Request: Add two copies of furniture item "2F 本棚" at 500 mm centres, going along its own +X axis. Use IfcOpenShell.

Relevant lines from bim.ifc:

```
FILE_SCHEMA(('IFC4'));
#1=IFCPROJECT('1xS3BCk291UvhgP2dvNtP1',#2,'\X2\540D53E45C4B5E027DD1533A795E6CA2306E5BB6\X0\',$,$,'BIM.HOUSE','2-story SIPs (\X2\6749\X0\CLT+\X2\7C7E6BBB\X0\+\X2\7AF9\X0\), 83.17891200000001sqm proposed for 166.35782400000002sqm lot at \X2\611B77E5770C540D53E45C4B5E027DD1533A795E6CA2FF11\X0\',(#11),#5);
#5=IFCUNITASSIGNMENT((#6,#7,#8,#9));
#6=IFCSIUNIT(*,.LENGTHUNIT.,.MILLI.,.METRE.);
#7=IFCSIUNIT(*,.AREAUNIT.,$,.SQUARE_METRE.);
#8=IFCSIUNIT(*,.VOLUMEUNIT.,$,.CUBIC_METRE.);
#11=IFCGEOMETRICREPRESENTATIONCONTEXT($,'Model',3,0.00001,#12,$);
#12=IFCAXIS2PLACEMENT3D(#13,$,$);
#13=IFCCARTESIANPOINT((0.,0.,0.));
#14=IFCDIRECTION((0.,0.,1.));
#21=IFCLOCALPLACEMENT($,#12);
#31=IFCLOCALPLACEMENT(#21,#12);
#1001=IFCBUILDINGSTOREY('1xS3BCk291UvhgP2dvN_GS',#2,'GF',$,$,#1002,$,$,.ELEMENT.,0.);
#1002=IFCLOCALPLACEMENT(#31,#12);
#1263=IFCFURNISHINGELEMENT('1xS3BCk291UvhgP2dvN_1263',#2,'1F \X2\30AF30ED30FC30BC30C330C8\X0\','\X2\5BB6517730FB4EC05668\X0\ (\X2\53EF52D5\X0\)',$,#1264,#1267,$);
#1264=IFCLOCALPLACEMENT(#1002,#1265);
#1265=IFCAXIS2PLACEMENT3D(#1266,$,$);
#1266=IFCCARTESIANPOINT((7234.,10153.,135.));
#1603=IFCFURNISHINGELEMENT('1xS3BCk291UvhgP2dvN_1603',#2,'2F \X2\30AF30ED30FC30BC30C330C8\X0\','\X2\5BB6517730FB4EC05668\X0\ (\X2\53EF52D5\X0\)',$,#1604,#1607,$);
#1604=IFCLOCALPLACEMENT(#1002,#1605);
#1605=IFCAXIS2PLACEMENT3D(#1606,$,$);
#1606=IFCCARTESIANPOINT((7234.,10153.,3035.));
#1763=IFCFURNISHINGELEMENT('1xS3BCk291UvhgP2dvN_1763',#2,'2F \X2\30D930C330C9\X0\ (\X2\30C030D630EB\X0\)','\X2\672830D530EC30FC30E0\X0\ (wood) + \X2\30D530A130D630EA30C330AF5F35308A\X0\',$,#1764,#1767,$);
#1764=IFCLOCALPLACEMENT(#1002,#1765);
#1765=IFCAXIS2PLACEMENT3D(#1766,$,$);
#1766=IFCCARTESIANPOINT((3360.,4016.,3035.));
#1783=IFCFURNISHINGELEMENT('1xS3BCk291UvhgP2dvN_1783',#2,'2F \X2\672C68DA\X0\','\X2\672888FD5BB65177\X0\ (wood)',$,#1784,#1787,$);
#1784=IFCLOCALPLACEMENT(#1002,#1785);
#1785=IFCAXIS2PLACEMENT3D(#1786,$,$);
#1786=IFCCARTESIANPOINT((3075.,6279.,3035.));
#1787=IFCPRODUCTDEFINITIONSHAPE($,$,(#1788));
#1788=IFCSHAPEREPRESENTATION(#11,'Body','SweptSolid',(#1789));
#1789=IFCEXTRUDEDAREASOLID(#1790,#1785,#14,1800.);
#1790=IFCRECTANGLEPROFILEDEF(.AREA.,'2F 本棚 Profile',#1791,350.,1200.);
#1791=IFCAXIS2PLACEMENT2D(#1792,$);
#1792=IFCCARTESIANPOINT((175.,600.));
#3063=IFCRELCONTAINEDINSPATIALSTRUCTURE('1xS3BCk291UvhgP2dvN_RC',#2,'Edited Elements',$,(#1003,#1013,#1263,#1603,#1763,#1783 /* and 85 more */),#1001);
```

```python
import ifcopenshell
import ifcopenshell.api.geometry
import ifcopenshell.api.root
import ifcopenshell.util.element
import ifcopenshell.util.placement

model = ifcopenshell.open("bim.ifc")


def reuse_history(source, copy):
    """copy_class also copies each property set's owner history, people and application; keep the originals."""
    for rel in copy.IsDefinedBy:
        if rel.is_a("IfcRelDefinesByProperties") and (history := rel.RelatingPropertyDefinition.OwnerHistory):
            rel.RelatingPropertyDefinition.OwnerHistory = source.OwnerHistory
            ifcopenshell.util.element.remove_deep2(model, history)


source = model.by_id(1783)
base = ifcopenshell.util.placement.get_local_placement(source.ObjectPlacement)
step = base[:3, 0] * 500.0

for i in range(1, 3):
    copy = ifcopenshell.api.root.copy_class(model, product=source)
    copy.Representation = ifcopenshell.util.element.copy_deep(
        model, source.Representation, exclude=["IfcGeometricRepresentationContext", "IfcRepresentationMap"]
    )
    reuse_history(source, copy)
    matrix = base.copy()
    matrix[:3, 3] += i * step
    print("added at", matrix[:3, 3].round(3) + 0.0)
    ifcopenshell.api.geometry.edit_object_placement(model, product=copy, matrix=matrix, is_si=False)

model.write("bim_edited.ifc")
```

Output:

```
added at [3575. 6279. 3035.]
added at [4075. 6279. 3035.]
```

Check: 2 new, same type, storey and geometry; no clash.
